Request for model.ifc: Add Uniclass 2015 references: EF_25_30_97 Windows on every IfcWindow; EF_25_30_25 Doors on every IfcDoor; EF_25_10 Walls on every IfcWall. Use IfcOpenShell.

First a look at what the model holds.

```python
import ifcopenshell

model = ifcopenshell.open("model.ifc")
print(model.schema)
print("classifications:", [c.Name for c in model.by_type("IfcClassification")])
for ifc_class in ("IfcDoor", "IfcRoof", "IfcStair", "IfcWall", "IfcWindow"):
    print(ifc_class, len(model.by_type(ifc_class)))
```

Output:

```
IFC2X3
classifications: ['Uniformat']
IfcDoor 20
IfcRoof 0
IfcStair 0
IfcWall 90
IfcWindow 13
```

```python
import ifcopenshell
import ifcopenshell.api.classification

model = ifcopenshell.open("model.ifc")

# IFC2X3 requires Source and Edition and has no link from the project to the system.
system = model.create_entity("IfcClassification", Source="NBS", Edition="2015", Name="Uniclass 2015")

codes = {
    "IfcWindow": ("EF_25_30_97", "Windows"),
    "IfcDoor": ("EF_25_30_25", "Doors"),
    "IfcWall": ("EF_25_10", "Walls"),
}
for ifc_class, (code, name) in codes.items():
    products = model.by_type(ifc_class)
    ifcopenshell.api.classification.add_reference(
        model, products=products, classification=system, identification=code, name=name
    )
    print(code, len(products))

model.write("model_edited.ifc")
```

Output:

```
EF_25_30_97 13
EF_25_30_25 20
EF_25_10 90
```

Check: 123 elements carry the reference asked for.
